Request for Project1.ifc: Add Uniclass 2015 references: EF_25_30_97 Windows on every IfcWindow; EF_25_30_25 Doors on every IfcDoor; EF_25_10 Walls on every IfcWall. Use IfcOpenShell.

First a look at what the model holds.

```python
import ifcopenshell

model = ifcopenshell.open("Project1.ifc")
print(model.schema)
print("classifications:", [c.Name for c in model.by_type("IfcClassification")])
for ifc_class in ("IfcDoor", "IfcRoof", "IfcStair", "IfcWall", "IfcWindow"):
    print(ifc_class, len(model.by_type(ifc_class)))
```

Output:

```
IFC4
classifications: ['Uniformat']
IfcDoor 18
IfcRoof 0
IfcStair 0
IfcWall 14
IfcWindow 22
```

```python
import ifcopenshell
import ifcopenshell.api.classification

model = ifcopenshell.open("Project1.ifc")

system = ifcopenshell.api.classification.add_classification(model, classification="Uniclass 2015")

codes = {
    "IfcWindow": ("EF_25_30_97", "Windows"),
    "IfcDoor": ("EF_25_30_25", "Doors"),
    "IfcWall": ("EF_25_10", "Walls"),
}
for ifc_class, (code, name) in codes.items():
    products = model.by_type(ifc_class)
    ifcopenshell.api.classification.add_reference(
        model, products=products, classification=system, identification=code, name=name
    )
    print(code, len(products))

model.write("Project1_rev.ifc")
```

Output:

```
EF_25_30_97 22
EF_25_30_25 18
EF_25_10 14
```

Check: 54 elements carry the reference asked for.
